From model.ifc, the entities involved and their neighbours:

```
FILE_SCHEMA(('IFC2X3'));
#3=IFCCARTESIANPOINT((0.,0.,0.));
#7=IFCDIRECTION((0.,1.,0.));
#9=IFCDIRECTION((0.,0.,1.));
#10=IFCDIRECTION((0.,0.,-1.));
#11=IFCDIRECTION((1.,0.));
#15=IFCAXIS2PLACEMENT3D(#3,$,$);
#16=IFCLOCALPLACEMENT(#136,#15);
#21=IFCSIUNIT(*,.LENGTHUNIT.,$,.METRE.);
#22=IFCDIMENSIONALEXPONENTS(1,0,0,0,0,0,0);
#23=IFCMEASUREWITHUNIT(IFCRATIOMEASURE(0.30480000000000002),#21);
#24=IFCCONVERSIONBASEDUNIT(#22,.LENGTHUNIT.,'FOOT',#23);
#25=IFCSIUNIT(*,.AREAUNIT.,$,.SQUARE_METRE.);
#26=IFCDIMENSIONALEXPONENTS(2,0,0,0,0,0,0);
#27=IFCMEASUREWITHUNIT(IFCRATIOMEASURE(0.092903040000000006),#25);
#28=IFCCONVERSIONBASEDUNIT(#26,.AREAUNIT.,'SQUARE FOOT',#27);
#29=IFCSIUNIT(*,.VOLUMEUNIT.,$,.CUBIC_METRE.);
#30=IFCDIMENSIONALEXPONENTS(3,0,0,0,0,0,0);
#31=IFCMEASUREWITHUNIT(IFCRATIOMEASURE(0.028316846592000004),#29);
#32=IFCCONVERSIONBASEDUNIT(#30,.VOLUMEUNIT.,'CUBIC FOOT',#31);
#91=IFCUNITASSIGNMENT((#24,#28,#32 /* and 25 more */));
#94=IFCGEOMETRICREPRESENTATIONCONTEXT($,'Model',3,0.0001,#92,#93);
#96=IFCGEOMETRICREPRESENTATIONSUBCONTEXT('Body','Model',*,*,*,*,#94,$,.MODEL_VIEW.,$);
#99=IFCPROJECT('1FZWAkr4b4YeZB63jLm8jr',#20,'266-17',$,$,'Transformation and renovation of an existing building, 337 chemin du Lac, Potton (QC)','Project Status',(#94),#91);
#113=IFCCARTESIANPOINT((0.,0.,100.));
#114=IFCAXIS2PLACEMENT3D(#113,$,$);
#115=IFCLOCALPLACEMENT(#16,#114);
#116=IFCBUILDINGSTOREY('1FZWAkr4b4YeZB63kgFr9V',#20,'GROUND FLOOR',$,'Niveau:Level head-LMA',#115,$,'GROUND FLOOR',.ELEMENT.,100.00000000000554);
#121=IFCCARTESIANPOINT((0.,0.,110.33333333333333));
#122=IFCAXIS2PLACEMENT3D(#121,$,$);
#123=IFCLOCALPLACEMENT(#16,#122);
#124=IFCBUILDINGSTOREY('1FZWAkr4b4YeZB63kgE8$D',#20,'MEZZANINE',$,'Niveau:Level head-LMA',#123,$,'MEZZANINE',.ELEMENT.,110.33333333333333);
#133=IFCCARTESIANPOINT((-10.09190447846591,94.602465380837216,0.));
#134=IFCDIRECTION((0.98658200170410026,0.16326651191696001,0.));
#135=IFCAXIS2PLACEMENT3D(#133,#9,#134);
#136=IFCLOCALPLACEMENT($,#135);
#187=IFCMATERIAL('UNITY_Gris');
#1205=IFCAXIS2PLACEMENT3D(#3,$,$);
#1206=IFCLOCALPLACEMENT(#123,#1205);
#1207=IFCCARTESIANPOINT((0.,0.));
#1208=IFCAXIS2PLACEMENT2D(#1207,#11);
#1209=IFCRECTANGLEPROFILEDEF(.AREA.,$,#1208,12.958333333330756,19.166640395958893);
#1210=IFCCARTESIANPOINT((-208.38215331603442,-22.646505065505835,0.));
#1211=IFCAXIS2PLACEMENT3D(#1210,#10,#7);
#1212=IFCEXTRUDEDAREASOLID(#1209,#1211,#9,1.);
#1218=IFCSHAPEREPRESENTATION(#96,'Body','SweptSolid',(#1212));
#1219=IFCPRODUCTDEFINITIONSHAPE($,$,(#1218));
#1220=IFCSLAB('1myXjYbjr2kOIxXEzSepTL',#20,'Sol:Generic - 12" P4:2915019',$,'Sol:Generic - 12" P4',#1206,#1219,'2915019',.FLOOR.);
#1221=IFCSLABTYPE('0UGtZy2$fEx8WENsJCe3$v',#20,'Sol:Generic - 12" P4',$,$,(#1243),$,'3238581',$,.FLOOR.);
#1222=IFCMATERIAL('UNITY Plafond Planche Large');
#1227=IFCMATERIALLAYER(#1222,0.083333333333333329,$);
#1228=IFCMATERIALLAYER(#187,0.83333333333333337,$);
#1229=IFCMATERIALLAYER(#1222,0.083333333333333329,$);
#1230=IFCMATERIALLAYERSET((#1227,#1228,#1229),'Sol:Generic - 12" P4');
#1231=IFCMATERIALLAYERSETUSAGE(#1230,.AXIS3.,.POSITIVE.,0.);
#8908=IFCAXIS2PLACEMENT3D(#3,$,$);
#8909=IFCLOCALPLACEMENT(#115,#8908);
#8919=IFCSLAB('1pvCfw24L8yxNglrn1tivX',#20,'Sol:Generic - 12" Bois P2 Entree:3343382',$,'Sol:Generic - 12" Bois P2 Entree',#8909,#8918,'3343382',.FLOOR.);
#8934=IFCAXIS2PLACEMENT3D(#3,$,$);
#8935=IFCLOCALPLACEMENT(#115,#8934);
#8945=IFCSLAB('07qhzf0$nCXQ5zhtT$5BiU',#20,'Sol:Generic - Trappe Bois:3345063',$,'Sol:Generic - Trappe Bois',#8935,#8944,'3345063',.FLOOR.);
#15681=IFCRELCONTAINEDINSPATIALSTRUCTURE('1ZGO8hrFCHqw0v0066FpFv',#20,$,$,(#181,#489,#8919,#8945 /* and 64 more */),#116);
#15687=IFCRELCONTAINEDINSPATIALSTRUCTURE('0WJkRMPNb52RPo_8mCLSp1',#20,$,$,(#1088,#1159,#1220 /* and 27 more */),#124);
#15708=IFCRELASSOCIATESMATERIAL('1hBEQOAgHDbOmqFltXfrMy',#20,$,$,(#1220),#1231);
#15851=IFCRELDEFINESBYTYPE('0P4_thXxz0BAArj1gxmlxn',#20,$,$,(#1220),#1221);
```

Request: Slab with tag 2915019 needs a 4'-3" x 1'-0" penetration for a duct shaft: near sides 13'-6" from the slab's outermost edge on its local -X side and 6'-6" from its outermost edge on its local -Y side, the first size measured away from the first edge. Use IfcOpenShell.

```python
import numpy as np
import ifcopenshell
import ifcopenshell.api.feature
import ifcopenshell.api.geometry
import ifcopenshell.api.root
import ifcopenshell.geom
import ifcopenshell.util.placement
import ifcopenshell.util.representation
import ifcopenshell.util.shape
import ifcopenshell.util.unit

model = ifcopenshell.open("model.ifc")
unit_scale = ifcopenshell.util.unit.calculate_unit_scale(model)
settings = ifcopenshell.geom.settings()


def volume(element):
    """Net volume in cubic metres, openings subtracted."""
    shape = ifcopenshell.geom.create_shape(settings, element)
    return ifcopenshell.util.shape.get_volume(shape.geometry)


slab = model.by_guid("1myXjYbjr2kOIxXEzSepTL")
before = volume(slab)

# Extent in the slab's own axes, in metres. The edges named are its -X and -Y sides.
slab_shape = ifcopenshell.geom.create_shape(settings, slab)
vertices = ifcopenshell.util.shape.get_vertices(slab_shape.geometry)
x_min, y_min, bottom = vertices.min(axis=0)
top = vertices[:, 2].max()

opening = ifcopenshell.api.root.create_entity(model, ifc_class="IfcOpeningElement", name="Duct shaft opening")
context = ifcopenshell.util.representation.get_context(model, "Model", "Body", "MODEL_VIEW")
width, depth = 1.2954, 0.3048
outline = [(0.0, 0.0), (width, 0.0), (width, depth), (0.0, depth), (0.0, 0.0)]
# Overshoot both faces by 50 mm so the cut is clean.
shape = ifcopenshell.api.geometry.add_slab_representation(
    model, context=context, depth=top - bottom + 0.1, polyline=outline
)
ifcopenshell.api.geometry.assign_representation(model, product=opening, representation=shape)

matrix = ifcopenshell.util.placement.get_local_placement(slab.ObjectPlacement)
matrix[:, 3] = matrix @ np.append(np.array([x_min + 4.1148, y_min + 1.9812, bottom - 0.05]) / unit_scale, 1.0)
ifcopenshell.api.geometry.edit_object_placement(model, product=opening, matrix=matrix, is_si=False)
ifcopenshell.api.feature.add_feature(model, feature=opening, element=slab)

after = volume(slab)

print(f"slab volume {before:.3f} -> {after:.3f} m3")

model.write("model_updated.ifc")
```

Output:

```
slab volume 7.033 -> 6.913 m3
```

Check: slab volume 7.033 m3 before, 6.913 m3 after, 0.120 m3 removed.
